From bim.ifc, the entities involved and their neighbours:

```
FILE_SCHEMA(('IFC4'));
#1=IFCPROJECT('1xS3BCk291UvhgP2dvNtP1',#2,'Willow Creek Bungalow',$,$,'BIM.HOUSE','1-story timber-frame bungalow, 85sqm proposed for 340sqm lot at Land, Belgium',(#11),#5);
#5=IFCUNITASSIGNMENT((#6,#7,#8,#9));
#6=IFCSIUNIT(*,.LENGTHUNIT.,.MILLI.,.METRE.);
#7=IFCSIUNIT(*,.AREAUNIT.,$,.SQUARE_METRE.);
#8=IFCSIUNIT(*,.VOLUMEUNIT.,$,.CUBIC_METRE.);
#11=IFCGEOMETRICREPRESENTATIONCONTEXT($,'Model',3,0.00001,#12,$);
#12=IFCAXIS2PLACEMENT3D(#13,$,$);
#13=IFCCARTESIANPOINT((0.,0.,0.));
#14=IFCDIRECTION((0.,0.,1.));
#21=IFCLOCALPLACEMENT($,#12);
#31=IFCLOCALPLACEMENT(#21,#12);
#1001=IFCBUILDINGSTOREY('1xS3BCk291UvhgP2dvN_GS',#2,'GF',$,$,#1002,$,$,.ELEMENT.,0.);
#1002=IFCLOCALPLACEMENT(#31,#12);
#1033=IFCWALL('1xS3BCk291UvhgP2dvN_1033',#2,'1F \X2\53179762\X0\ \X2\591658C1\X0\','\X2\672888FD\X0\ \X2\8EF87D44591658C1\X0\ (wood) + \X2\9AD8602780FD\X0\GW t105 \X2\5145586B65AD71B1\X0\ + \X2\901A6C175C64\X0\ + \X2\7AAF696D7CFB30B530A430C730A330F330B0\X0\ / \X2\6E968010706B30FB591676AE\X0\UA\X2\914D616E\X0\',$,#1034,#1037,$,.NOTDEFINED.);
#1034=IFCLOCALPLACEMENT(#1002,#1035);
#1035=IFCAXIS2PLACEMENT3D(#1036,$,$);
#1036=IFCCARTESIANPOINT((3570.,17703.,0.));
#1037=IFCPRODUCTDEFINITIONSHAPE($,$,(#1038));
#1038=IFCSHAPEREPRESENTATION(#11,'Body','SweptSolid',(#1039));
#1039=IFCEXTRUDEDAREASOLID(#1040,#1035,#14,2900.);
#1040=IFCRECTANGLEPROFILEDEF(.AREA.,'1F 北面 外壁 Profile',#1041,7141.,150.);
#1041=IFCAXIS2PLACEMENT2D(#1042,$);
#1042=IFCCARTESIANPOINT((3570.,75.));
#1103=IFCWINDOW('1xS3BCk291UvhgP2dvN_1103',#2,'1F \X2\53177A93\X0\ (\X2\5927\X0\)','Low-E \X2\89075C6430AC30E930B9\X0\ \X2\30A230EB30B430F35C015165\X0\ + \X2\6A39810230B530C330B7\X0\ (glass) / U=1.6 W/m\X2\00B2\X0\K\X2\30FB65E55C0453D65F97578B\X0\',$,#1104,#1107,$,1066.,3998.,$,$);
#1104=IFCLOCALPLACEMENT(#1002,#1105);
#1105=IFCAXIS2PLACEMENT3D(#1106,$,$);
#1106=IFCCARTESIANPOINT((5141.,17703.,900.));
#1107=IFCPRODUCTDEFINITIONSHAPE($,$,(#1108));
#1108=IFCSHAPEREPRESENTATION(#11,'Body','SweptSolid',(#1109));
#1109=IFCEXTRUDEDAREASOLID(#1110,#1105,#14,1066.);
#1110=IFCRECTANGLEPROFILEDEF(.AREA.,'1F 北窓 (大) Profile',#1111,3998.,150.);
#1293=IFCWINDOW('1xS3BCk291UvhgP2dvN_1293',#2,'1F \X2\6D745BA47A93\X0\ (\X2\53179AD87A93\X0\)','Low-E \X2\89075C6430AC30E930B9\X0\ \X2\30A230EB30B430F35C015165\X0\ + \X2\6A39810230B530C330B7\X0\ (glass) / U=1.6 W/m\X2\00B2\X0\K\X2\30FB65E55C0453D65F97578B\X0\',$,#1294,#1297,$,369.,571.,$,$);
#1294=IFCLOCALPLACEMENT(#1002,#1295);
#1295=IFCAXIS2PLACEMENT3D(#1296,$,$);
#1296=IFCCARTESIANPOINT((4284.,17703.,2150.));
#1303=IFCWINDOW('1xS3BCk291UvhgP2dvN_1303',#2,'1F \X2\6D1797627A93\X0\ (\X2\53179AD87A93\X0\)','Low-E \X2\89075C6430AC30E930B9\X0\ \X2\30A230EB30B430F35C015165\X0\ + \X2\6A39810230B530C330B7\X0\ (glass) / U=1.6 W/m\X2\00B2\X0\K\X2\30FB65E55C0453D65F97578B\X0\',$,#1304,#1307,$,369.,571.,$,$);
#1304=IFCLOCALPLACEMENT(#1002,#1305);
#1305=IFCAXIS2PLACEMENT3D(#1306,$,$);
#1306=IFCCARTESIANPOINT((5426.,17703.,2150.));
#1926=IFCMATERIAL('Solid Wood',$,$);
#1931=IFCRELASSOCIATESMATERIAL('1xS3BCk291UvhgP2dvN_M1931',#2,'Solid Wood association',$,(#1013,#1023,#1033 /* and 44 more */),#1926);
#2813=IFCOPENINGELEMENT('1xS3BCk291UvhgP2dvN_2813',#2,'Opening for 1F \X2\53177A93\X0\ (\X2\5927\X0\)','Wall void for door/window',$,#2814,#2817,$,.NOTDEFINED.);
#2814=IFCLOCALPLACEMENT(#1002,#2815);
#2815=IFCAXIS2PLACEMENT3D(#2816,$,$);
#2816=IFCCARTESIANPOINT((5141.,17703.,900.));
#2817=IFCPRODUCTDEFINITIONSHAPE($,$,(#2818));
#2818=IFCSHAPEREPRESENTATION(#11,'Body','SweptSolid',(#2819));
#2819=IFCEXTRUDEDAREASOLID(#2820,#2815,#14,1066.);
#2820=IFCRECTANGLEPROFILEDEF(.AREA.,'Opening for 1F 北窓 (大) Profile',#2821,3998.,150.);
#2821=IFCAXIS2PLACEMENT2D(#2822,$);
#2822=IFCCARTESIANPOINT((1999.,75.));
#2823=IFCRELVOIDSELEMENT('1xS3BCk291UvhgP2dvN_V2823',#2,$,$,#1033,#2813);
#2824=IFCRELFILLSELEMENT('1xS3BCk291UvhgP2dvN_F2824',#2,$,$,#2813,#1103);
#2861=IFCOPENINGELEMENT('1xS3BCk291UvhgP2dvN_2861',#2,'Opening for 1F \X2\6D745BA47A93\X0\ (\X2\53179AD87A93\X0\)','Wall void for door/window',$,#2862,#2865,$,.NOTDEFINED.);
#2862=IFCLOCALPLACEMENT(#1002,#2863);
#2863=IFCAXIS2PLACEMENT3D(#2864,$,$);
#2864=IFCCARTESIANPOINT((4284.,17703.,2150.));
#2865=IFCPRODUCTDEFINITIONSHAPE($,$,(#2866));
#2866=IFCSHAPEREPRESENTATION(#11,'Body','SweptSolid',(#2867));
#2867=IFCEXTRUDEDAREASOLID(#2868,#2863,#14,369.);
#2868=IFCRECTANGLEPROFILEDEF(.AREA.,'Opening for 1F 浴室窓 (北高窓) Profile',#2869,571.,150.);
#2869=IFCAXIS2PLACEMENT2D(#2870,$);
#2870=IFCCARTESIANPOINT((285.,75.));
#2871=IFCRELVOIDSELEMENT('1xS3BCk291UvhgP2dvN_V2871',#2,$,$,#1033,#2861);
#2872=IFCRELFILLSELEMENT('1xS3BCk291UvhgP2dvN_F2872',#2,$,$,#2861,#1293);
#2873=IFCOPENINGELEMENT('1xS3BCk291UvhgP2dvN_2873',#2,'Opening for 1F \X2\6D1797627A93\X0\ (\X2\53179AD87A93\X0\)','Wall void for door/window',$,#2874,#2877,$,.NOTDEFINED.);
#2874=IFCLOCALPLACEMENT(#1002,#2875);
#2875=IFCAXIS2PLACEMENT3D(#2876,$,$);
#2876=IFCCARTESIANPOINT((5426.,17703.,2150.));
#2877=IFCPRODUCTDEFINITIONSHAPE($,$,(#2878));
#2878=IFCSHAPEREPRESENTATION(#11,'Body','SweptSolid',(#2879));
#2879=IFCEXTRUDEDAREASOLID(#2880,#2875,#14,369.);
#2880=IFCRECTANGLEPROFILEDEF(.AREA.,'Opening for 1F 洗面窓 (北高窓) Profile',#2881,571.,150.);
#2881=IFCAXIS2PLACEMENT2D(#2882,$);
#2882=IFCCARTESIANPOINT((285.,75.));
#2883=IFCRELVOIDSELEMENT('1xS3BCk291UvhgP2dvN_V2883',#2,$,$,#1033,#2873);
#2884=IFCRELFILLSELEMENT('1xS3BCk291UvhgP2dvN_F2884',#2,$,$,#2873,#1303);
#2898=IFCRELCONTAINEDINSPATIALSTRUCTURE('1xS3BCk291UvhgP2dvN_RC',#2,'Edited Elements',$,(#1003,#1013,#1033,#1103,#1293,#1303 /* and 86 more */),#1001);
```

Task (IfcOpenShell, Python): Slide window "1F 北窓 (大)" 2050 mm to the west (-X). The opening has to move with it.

```python
import ifcopenshell
import ifcopenshell.api.geometry
import ifcopenshell.util.placement
import ifcopenshell.util.unit

model = ifcopenshell.open("bim.ifc")
unit_scale = ifcopenshell.util.unit.calculate_unit_scale(model)

window = model.by_guid("1xS3BCk291UvhgP2dvN_1103")
opening = window.FillsVoids[0].RelatingOpeningElement
wall = opening.VoidsElements[0].RelatingBuildingElement

wall_matrix = ifcopenshell.util.placement.get_local_placement(wall.ObjectPlacement)
shift = wall_matrix[:3, 0] * -2.05 / unit_scale
before = ifcopenshell.util.placement.get_local_placement(window.ObjectPlacement)[:3, 3].copy()

# The window is not placed relative to its opening, so move both.
for product in (opening, window):
    matrix = ifcopenshell.util.placement.get_local_placement(product.ObjectPlacement)
    matrix[:3, 3] += shift
    ifcopenshell.api.geometry.edit_object_placement(model, product=product, matrix=matrix, is_si=False)

after = ifcopenshell.util.placement.get_local_placement(window.ObjectPlacement)[:3, 3]
print("window moved by", (after - before).round(3) + 0.0)

model.write("bim-out.ifc")
```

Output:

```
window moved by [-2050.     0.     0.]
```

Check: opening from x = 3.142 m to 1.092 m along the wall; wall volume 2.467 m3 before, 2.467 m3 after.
